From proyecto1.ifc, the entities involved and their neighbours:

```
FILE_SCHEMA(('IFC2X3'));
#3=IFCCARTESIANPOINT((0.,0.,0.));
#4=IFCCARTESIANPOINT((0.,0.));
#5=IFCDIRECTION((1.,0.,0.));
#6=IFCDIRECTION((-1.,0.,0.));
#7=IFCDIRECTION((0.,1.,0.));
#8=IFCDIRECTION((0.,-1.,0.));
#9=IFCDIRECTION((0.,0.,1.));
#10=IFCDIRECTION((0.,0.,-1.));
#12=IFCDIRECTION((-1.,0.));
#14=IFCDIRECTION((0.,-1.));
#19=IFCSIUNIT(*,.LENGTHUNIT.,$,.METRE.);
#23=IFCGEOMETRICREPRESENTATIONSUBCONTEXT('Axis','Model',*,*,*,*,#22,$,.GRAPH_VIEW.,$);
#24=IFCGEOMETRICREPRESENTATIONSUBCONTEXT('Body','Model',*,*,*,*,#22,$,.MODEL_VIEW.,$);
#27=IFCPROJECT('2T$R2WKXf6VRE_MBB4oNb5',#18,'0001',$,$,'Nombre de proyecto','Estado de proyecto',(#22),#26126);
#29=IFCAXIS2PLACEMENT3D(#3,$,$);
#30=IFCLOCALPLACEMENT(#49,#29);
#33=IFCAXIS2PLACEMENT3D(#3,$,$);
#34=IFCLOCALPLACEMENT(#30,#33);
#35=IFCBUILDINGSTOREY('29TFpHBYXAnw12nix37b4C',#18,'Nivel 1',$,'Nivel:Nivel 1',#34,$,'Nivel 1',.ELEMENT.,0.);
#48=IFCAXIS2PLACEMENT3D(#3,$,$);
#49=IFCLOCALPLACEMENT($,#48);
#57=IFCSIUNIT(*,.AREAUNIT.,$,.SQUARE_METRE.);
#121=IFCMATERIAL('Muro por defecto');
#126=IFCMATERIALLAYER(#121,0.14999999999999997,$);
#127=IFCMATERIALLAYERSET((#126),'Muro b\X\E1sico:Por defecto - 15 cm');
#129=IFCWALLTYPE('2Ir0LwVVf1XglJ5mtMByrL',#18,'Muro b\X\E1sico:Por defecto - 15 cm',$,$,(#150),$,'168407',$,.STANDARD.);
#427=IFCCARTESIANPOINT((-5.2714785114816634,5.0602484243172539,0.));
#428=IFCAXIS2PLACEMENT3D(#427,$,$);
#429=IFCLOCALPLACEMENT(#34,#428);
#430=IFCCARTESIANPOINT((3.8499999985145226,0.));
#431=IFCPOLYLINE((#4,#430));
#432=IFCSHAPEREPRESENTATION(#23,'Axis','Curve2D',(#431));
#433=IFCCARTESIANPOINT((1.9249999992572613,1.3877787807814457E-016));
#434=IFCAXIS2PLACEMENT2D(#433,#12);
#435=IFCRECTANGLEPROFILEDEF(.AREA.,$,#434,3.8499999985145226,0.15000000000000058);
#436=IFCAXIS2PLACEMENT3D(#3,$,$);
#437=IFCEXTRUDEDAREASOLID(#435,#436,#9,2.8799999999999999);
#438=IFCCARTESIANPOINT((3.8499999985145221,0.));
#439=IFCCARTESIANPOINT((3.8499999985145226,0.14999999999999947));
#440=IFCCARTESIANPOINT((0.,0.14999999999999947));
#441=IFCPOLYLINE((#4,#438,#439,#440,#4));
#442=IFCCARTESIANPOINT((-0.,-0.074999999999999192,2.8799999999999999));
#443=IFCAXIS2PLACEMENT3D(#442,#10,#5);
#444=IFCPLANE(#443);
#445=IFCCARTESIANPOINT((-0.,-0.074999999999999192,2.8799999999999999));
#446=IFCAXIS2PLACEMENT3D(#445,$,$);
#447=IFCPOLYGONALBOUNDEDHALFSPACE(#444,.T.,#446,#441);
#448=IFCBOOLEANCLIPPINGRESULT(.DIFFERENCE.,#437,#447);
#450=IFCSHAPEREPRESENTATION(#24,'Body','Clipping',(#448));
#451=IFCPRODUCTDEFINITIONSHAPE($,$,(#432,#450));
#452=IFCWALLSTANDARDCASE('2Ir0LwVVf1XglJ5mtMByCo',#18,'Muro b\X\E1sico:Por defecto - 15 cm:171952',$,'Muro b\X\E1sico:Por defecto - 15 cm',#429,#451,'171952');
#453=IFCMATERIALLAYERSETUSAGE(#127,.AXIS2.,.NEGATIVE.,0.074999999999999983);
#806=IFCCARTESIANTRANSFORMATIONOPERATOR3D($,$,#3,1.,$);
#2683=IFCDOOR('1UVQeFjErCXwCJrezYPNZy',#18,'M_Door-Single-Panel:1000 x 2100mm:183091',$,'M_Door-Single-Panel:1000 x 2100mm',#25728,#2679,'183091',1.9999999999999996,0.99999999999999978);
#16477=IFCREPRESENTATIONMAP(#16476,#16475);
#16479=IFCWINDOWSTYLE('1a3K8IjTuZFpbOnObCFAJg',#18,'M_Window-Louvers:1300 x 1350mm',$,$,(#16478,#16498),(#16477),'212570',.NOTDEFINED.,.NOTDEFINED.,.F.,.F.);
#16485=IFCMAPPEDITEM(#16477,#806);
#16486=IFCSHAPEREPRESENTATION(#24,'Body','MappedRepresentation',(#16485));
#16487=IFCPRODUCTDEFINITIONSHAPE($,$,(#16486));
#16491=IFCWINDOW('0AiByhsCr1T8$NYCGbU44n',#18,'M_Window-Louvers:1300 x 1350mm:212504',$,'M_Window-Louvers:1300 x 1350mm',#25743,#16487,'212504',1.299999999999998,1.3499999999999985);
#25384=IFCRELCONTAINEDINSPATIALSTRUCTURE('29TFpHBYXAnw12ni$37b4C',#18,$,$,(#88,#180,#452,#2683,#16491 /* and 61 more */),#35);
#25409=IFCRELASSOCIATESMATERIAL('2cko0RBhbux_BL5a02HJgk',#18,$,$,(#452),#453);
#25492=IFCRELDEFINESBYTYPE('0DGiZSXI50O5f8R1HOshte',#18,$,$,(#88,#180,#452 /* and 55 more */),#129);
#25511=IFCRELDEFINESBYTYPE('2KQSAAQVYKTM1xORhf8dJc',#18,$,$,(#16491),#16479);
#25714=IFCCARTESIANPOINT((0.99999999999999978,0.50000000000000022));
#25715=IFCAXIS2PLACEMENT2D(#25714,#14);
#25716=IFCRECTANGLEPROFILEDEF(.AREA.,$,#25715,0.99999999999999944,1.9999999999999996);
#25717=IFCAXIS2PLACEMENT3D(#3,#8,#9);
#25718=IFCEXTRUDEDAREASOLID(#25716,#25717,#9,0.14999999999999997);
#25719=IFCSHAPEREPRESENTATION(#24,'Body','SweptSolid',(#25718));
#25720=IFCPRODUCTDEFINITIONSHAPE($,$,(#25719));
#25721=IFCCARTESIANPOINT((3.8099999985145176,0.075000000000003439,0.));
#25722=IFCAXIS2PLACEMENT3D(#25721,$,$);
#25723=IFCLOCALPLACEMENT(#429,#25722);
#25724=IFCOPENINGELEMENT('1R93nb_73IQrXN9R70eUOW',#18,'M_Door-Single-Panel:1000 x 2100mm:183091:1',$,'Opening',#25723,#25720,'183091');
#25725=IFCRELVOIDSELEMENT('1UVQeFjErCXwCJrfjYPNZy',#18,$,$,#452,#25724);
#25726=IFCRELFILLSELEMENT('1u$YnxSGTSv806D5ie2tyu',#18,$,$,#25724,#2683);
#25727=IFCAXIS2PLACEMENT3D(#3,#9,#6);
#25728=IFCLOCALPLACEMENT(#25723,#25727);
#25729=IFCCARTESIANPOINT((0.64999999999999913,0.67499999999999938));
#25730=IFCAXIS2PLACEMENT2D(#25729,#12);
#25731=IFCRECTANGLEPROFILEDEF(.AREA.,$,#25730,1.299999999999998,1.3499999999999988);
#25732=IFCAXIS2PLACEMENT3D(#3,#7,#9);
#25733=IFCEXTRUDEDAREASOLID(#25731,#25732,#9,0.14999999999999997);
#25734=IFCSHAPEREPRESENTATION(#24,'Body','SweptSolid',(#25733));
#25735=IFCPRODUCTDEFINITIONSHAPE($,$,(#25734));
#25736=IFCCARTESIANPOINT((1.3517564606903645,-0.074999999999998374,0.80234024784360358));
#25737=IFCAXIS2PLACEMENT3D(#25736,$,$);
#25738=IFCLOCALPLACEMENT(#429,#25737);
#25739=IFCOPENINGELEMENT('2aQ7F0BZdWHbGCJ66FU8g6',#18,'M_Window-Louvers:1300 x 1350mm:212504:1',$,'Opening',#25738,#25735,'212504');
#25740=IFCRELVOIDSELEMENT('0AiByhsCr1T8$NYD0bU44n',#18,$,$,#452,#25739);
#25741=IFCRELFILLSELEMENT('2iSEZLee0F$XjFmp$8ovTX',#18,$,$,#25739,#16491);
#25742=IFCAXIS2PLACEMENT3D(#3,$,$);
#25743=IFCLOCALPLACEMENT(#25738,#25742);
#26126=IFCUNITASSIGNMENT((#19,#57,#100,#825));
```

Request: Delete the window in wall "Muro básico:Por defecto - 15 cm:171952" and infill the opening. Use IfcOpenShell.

```python
import ifcopenshell
import ifcopenshell.api.feature
import ifcopenshell.api.root
import ifcopenshell.geom
import ifcopenshell.util.shape

model = ifcopenshell.open("proyecto1.ifc")
settings = ifcopenshell.geom.settings()


def volume(element):
    """Net volume in cubic metres, openings subtracted."""
    shape = ifcopenshell.geom.create_shape(settings, element)
    return ifcopenshell.util.shape.get_volume(shape.geometry)


window = model.by_id(16491)
opening = window.FillsVoids[0].RelatingOpeningElement
wall = opening.VoidsElements[0].RelatingBuildingElement
before = volume(wall)

ifcopenshell.api.root.remove_product(model, product=window)
ifcopenshell.api.feature.remove_feature(model, feature=opening)

after = volume(wall)

print(f"wall volume {before:.3f} -> {after:.3f} m3")

model.write("proyecto1-out.ifc")
```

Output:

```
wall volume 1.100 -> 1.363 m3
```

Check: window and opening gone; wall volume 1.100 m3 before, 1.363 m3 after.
